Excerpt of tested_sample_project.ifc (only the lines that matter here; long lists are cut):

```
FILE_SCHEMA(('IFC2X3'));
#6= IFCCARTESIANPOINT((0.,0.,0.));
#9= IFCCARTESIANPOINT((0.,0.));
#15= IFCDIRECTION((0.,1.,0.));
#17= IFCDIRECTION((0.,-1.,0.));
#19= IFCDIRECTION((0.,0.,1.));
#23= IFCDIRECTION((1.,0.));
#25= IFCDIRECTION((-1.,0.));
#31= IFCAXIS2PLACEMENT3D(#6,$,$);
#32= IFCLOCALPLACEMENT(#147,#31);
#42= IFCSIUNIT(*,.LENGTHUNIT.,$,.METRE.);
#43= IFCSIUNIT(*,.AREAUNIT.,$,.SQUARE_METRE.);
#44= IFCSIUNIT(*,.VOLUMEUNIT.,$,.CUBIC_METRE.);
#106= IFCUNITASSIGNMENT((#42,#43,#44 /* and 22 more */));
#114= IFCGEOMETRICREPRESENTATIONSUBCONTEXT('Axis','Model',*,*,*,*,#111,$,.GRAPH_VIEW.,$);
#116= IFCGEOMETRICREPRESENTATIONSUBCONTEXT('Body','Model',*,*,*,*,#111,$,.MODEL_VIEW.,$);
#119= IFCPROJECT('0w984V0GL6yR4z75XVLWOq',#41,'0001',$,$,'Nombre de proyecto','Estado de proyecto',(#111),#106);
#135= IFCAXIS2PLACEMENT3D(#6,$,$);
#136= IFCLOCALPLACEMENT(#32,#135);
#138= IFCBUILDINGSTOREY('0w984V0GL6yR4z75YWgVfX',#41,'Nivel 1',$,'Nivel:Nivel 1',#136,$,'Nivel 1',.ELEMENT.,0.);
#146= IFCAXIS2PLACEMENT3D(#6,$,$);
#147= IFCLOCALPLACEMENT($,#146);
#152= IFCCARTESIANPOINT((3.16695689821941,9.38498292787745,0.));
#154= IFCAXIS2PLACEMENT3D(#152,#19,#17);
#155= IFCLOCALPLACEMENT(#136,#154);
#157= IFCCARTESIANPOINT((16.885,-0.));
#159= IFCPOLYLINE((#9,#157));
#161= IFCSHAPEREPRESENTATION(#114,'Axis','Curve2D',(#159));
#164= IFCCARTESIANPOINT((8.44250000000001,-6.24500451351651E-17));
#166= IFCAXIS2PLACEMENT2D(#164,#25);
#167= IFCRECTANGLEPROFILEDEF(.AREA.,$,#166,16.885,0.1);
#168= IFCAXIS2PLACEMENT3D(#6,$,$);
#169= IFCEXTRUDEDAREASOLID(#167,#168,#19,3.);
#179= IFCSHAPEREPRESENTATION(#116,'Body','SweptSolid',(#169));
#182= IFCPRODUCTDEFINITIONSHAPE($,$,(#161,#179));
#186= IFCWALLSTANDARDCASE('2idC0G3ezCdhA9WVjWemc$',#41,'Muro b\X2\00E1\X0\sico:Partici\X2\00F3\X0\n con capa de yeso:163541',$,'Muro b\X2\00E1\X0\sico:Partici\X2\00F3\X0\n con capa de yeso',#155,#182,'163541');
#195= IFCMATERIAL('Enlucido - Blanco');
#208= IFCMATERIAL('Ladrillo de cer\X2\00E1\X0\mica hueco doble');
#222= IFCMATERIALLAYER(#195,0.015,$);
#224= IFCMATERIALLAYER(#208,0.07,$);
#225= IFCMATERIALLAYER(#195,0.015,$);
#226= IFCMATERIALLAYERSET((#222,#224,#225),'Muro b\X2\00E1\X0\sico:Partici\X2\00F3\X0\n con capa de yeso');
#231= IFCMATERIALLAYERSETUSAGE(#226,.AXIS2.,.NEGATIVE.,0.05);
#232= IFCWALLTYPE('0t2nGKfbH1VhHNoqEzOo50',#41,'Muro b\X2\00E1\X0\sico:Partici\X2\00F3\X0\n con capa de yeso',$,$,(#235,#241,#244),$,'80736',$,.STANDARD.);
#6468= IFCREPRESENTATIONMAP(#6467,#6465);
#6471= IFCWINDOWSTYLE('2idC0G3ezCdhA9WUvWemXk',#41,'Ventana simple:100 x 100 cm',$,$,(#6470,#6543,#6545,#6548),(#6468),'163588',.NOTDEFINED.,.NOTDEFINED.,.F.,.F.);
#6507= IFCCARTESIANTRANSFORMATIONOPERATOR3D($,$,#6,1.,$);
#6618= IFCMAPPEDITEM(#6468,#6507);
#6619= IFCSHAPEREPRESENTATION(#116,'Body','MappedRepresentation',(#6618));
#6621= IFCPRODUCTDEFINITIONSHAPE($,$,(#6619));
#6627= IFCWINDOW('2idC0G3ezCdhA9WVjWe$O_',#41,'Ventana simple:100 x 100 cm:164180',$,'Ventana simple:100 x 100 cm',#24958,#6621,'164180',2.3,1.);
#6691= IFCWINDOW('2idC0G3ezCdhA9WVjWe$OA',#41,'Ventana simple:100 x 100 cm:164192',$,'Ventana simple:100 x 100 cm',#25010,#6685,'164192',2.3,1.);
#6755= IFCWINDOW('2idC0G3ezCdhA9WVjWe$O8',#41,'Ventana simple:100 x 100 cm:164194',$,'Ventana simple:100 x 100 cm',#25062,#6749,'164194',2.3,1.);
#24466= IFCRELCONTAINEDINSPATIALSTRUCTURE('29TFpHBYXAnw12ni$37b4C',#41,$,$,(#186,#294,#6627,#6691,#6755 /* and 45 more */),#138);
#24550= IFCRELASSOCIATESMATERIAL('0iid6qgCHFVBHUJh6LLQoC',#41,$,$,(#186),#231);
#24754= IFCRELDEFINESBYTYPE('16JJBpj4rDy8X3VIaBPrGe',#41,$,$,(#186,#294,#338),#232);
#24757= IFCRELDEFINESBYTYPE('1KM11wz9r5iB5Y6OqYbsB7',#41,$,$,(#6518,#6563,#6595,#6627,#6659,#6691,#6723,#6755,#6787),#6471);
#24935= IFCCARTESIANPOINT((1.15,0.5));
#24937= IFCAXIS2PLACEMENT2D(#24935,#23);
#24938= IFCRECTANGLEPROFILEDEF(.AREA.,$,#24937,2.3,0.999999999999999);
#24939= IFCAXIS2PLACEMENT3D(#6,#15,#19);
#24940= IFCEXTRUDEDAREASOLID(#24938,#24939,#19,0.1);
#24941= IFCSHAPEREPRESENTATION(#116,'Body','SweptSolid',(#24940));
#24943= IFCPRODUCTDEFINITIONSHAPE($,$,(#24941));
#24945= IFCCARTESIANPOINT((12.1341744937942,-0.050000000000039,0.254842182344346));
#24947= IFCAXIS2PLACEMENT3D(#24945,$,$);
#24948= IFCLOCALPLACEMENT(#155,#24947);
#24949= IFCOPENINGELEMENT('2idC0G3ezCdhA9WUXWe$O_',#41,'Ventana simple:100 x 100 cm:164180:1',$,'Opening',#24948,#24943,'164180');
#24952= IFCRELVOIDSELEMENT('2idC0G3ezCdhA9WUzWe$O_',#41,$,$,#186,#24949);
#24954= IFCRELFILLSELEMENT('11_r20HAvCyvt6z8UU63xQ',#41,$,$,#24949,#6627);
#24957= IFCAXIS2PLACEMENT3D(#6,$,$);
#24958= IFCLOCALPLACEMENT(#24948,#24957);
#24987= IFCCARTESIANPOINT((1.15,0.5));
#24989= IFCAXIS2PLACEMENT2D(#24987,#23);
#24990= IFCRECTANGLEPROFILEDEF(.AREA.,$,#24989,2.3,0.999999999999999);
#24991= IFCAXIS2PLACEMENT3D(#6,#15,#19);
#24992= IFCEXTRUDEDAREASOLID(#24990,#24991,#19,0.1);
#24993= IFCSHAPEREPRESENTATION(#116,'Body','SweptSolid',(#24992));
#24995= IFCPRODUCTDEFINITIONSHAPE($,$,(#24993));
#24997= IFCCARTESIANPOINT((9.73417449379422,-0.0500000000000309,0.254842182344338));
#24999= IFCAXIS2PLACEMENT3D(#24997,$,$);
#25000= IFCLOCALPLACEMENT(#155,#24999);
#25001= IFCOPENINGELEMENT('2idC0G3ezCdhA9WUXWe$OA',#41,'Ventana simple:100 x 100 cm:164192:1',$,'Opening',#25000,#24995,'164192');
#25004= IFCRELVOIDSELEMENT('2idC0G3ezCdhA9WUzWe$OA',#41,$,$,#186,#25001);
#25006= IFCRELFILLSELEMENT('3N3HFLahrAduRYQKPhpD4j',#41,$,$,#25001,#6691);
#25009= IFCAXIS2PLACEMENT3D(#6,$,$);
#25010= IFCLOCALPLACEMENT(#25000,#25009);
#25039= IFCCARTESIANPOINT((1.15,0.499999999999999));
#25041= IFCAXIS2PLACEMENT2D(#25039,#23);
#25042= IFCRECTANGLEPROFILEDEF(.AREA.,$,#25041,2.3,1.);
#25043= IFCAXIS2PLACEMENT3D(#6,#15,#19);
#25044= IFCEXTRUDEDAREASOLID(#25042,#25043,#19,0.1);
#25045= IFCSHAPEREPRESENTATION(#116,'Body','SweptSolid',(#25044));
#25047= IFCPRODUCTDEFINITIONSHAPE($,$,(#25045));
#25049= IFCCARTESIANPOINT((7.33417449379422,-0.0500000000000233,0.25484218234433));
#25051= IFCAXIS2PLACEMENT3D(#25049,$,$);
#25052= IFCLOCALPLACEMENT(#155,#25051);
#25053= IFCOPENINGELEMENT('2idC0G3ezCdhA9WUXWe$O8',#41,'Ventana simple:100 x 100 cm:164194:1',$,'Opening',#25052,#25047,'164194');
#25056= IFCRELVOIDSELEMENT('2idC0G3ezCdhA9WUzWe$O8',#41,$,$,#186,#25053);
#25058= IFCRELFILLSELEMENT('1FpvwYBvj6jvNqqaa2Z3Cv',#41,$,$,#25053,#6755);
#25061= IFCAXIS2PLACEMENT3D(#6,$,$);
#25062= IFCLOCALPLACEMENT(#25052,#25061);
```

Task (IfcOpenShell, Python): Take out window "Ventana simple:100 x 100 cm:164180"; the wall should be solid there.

```python
import ifcopenshell
import ifcopenshell.api.feature
import ifcopenshell.api.root
import ifcopenshell.geom
import ifcopenshell.util.shape

model = ifcopenshell.open("tested_sample_project.ifc")
settings = ifcopenshell.geom.settings()


def volume(element):
    """Net volume in cubic metres, openings subtracted."""
    shape = ifcopenshell.geom.create_shape(settings, element)
    return ifcopenshell.util.shape.get_volume(shape.geometry)


window = model.by_id(6627)
opening = window.FillsVoids[0].RelatingOpeningElement
wall = opening.VoidsElements[0].RelatingBuildingElement
before = volume(wall)

ifcopenshell.api.root.remove_product(model, product=window)
ifcopenshell.api.feature.remove_feature(model, feature=opening)

after = volume(wall)

print(f"wall volume {before:.3f} -> {after:.3f} m3")

model.write("tested_sample_project_edited.ifc")
```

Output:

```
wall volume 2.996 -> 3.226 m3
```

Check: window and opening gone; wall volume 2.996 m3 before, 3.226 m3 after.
